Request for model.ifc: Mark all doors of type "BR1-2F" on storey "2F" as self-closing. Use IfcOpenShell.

First a look at what the model holds.

```python
import ifcopenshell
import ifcopenshell.util.element

model = ifcopenshell.open("model.ifc")
print(model.schema)
storey = next(s for s in model.by_type("IfcBuildingStorey") if s.Name == "2F")
doors = [e for e in ifcopenshell.util.element.get_decomposition(storey) if e.is_a("IfcDoor")]
seen = {}
for e in doors:
    element_type = ifcopenshell.util.element.get_type(e)
    key = (element_type.Name if element_type != e and element_type else None, ifcopenshell.util.element.get_pset(e, "Pset_DoorCommon", "SelfClosing"))
    seen[key] = seen.get(key, 0) + 1
for (name, value), count in sorted(seen.items(), key=str):
    print(count, "x", name, "|", value)
```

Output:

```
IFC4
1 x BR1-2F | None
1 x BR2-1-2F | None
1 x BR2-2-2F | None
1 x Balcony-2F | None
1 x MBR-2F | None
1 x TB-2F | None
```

```python
import ifcopenshell
import ifcopenshell.api.pset
import ifcopenshell.util.element

model = ifcopenshell.open("model.ifc")

storey = next(s for s in model.by_type("IfcBuildingStorey") if s.Name == "2F")
doors = [e for e in ifcopenshell.util.element.get_decomposition(storey) if e.is_a("IfcDoor")]

count = 0
for e in doors:
    element_type = ifcopenshell.util.element.get_type(e)
    if element_type in (None, e) or element_type.Name != "BR1-2F":
        continue
    # add_pset returns the element's existing set when there is one.
    pset = ifcopenshell.api.pset.add_pset(model, product=e, name="Pset_DoorCommon")
    ifcopenshell.api.pset.edit_pset(model, pset=pset, properties={"SelfClosing": True})
    count += 1

print(count, "doors updated")

model.write("model-out.ifc")
```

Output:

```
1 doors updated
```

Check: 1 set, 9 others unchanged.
